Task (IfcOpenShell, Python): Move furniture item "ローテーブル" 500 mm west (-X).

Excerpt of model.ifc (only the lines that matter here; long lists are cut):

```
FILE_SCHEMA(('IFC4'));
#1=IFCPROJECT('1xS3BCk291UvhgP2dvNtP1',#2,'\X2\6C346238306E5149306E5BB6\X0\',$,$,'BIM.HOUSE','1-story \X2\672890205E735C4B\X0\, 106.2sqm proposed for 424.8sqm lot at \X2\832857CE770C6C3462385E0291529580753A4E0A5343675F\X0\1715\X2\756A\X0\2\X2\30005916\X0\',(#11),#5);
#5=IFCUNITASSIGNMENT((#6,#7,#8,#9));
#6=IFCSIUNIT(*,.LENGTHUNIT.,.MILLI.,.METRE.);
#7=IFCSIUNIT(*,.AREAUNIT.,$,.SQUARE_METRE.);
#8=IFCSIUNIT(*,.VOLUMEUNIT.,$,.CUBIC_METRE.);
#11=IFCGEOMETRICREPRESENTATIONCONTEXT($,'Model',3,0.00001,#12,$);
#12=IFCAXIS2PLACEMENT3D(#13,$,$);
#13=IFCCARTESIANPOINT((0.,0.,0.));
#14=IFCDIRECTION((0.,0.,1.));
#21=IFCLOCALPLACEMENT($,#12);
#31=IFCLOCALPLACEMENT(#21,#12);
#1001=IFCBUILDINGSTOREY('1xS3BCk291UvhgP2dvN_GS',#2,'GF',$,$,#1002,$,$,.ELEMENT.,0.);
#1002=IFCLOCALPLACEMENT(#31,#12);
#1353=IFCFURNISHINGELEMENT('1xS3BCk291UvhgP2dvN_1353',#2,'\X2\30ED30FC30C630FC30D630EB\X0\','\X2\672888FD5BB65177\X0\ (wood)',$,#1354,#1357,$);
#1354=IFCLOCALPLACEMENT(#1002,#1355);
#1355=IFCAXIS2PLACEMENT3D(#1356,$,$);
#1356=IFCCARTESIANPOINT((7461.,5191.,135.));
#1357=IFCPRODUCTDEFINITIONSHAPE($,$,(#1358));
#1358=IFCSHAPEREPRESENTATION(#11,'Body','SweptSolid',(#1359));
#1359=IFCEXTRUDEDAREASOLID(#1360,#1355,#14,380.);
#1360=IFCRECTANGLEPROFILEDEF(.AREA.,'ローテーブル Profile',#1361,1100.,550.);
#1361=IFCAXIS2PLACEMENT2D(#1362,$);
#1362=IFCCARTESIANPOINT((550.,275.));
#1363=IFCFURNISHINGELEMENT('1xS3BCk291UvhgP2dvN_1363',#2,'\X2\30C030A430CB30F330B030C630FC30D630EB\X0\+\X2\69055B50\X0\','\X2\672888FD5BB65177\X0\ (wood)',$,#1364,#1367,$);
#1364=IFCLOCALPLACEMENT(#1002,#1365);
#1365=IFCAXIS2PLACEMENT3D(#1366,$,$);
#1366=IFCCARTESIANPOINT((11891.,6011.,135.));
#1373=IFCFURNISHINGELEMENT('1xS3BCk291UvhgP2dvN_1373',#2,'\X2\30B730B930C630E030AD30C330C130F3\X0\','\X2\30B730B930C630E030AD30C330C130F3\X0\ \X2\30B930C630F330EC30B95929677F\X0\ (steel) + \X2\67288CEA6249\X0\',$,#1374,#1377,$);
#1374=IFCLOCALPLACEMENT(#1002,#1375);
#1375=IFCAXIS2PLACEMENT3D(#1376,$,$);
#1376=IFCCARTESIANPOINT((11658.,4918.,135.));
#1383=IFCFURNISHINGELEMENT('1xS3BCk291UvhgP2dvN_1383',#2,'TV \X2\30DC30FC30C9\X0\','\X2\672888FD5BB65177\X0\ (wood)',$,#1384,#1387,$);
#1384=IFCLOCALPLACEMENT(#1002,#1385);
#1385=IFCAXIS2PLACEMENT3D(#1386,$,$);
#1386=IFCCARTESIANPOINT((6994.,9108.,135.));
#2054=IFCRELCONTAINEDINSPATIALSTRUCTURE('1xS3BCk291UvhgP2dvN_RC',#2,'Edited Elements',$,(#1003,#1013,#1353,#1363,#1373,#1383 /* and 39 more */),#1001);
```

```python
import ifcopenshell
import ifcopenshell.api.geometry
import ifcopenshell.util.placement

model = ifcopenshell.open("model.ifc")

item = model.by_guid("1xS3BCk291UvhgP2dvN_1353")
matrix = ifcopenshell.util.placement.get_local_placement(item.ObjectPlacement)
matrix[0, 3] -= 500.0
ifcopenshell.api.geometry.edit_object_placement(model, product=item, matrix=matrix, is_si=False)

print(ifcopenshell.util.placement.get_local_placement(item.ObjectPlacement).round(3) + 0.0)

model.write("model-out.ifc")
```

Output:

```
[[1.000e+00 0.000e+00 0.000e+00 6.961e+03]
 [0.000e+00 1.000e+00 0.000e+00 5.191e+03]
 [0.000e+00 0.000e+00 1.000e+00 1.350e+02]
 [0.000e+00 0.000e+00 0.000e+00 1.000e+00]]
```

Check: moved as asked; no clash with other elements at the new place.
